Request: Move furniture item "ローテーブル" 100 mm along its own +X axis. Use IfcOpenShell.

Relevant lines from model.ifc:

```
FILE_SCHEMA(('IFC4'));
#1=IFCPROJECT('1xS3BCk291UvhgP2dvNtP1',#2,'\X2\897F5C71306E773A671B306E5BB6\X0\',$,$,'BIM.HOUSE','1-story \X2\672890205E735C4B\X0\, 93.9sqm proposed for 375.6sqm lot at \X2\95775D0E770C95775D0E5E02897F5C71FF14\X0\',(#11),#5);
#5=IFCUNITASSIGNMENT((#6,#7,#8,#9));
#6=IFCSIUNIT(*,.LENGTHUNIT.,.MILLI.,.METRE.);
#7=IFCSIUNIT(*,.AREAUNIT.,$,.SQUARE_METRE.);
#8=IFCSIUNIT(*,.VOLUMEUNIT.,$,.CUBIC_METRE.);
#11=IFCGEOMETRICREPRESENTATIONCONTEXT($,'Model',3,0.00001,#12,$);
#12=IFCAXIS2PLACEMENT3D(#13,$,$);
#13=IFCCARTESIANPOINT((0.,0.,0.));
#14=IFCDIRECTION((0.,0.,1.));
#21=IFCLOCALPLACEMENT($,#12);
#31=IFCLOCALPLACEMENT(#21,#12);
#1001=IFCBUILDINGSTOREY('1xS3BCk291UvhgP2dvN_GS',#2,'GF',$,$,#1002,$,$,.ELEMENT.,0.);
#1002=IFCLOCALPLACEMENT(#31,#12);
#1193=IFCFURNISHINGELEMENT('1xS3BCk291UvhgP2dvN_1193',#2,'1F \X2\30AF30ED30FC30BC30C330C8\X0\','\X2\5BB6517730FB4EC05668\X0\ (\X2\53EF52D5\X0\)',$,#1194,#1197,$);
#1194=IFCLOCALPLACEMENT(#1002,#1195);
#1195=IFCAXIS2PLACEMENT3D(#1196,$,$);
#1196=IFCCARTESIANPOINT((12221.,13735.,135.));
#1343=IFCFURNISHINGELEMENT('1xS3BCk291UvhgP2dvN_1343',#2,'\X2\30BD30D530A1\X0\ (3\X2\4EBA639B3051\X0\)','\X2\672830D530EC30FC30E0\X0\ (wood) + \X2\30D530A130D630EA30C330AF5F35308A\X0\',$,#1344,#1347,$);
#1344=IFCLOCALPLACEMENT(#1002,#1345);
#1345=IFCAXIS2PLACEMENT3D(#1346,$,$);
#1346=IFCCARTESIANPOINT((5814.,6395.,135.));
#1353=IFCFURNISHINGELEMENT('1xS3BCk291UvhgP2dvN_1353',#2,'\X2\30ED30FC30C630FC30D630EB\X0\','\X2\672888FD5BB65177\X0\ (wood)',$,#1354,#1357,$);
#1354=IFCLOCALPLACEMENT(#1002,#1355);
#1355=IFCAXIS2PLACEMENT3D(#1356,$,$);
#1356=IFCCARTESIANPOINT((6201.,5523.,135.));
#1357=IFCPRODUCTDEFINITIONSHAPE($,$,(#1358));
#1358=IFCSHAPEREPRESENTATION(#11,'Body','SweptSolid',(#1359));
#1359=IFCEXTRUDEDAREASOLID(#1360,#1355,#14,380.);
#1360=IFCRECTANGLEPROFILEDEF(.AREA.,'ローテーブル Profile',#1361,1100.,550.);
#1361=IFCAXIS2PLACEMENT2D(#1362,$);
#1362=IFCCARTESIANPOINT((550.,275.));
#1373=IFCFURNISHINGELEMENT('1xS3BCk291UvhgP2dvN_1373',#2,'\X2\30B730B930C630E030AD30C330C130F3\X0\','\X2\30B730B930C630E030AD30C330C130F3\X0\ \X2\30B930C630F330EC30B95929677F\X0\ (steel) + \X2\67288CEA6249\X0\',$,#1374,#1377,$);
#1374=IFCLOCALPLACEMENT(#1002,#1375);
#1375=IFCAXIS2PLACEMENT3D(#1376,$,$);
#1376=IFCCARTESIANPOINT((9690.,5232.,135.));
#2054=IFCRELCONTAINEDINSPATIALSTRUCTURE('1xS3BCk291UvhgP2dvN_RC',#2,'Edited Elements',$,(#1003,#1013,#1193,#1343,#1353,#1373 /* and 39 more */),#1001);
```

```python
import ifcopenshell
import ifcopenshell.api.geometry
import ifcopenshell.util.placement

model = ifcopenshell.open("model.ifc")

item = model.by_id(1353)
matrix = ifcopenshell.util.placement.get_local_placement(item.ObjectPlacement)
matrix[:3, 3] += matrix[:3, 0] * 100.0
ifcopenshell.api.geometry.edit_object_placement(model, product=item, matrix=matrix, is_si=False)

print(ifcopenshell.util.placement.get_local_placement(item.ObjectPlacement).round(3) + 0.0)

model.write("model-out.ifc")
```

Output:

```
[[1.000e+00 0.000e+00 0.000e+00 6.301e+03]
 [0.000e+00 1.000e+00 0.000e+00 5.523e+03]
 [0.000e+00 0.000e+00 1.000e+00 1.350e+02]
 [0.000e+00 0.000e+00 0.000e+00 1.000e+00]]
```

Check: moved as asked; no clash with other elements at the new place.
